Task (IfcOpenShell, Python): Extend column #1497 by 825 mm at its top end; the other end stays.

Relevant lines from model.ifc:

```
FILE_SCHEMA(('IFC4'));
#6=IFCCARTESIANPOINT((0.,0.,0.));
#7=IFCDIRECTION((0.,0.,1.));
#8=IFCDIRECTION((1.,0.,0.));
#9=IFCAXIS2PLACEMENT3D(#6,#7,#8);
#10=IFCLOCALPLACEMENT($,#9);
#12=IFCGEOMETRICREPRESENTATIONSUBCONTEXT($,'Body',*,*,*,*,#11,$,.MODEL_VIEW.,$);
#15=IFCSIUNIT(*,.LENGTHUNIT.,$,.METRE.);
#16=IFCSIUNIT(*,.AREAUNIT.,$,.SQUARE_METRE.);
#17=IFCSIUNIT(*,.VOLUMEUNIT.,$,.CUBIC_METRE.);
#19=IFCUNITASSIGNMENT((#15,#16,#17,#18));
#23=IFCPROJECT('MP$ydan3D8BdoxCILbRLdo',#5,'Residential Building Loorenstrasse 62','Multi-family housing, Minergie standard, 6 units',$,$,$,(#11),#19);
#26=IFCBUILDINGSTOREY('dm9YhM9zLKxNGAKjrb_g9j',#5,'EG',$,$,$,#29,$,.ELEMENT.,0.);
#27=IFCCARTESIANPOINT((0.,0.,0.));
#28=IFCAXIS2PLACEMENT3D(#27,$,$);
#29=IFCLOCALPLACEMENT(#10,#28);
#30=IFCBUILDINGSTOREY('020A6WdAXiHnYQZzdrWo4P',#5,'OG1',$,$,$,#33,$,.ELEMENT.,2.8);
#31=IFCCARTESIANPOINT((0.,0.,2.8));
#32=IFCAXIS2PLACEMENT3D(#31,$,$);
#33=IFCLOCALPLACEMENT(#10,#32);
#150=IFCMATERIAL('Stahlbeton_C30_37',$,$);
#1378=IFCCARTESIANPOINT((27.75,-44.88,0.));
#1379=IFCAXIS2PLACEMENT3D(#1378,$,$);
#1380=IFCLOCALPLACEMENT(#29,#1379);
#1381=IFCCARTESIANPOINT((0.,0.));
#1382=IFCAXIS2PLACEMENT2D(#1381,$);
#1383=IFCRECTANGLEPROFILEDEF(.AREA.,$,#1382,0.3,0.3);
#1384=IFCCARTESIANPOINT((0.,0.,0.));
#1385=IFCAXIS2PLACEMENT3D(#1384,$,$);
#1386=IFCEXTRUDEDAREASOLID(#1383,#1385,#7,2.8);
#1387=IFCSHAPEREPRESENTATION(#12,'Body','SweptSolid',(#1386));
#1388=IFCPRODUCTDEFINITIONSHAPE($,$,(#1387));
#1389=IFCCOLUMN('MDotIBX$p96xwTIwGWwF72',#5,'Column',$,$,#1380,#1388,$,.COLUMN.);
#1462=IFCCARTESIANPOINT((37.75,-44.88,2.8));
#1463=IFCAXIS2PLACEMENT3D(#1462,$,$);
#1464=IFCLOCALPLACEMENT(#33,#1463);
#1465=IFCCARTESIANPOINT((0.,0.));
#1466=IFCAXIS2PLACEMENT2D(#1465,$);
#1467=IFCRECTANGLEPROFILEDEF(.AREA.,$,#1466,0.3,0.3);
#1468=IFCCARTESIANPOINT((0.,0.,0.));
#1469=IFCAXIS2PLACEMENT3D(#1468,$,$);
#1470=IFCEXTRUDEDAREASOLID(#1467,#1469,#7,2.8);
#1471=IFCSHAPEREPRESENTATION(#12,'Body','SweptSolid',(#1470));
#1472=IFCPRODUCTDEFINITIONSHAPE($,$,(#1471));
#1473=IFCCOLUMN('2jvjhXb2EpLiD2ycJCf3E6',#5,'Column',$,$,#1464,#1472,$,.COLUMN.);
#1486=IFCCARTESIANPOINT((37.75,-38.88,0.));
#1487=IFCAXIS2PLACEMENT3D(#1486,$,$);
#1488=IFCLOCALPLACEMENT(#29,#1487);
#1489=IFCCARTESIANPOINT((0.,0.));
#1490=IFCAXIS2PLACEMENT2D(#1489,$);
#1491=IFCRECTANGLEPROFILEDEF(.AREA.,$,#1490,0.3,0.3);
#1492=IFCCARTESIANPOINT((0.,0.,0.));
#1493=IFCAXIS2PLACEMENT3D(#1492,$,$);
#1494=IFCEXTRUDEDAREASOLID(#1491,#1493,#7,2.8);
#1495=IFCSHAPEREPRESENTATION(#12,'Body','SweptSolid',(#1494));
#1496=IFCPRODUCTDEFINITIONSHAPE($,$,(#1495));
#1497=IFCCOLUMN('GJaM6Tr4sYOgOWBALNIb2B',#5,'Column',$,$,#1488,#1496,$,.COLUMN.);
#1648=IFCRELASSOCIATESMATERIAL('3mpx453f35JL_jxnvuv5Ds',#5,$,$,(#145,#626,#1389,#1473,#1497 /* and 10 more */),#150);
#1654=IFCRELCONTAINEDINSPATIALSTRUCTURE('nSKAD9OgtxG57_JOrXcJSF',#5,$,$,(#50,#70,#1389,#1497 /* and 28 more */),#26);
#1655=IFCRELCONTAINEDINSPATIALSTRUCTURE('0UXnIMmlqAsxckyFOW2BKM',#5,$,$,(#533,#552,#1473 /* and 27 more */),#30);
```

```python
import ifcopenshell

model = ifcopenshell.open("model.ifc")

member = model.by_guid("GJaM6Tr4sYOgOWBALNIb2B")
change = 0.825

# The extrusion runs towards the end named, so only its depth changes.
body = next(r for r in member.Representation.Representations if r.RepresentationIdentifier == "Body")
solid = body.Items[0]
old_length = solid.Depth
solid.Depth += change

print(f"length {old_length:g} -> {solid.Depth:g}")

model.write("model_rev.ifc")
```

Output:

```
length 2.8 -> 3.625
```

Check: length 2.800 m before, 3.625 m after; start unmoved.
